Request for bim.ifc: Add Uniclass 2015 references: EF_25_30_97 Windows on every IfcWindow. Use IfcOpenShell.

First a look at what the model holds.

```python
import ifcopenshell

model = ifcopenshell.open("bim.ifc")
print(model.schema)
print("classifications:", [c.Name for c in model.by_type("IfcClassification")])
for ifc_class in ("IfcDoor", "IfcRoof", "IfcStair", "IfcWall", "IfcWindow"):
    print(ifc_class, len(model.by_type(ifc_class)))
```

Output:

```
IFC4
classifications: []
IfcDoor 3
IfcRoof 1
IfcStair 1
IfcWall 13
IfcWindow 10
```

```python
import ifcopenshell
import ifcopenshell.api.classification

model = ifcopenshell.open("bim.ifc")

system = ifcopenshell.api.classification.add_classification(model, classification="Uniclass 2015")

codes = {
    "IfcWindow": ("EF_25_30_97", "Windows"),
}
for ifc_class, (code, name) in codes.items():
    products = model.by_type(ifc_class)
    ifcopenshell.api.classification.add_reference(
        model, products=products, classification=system, identification=code, name=name
    )
    print(code, len(products))

model.write("bim_edited.ifc")
```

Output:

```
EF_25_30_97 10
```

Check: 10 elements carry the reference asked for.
